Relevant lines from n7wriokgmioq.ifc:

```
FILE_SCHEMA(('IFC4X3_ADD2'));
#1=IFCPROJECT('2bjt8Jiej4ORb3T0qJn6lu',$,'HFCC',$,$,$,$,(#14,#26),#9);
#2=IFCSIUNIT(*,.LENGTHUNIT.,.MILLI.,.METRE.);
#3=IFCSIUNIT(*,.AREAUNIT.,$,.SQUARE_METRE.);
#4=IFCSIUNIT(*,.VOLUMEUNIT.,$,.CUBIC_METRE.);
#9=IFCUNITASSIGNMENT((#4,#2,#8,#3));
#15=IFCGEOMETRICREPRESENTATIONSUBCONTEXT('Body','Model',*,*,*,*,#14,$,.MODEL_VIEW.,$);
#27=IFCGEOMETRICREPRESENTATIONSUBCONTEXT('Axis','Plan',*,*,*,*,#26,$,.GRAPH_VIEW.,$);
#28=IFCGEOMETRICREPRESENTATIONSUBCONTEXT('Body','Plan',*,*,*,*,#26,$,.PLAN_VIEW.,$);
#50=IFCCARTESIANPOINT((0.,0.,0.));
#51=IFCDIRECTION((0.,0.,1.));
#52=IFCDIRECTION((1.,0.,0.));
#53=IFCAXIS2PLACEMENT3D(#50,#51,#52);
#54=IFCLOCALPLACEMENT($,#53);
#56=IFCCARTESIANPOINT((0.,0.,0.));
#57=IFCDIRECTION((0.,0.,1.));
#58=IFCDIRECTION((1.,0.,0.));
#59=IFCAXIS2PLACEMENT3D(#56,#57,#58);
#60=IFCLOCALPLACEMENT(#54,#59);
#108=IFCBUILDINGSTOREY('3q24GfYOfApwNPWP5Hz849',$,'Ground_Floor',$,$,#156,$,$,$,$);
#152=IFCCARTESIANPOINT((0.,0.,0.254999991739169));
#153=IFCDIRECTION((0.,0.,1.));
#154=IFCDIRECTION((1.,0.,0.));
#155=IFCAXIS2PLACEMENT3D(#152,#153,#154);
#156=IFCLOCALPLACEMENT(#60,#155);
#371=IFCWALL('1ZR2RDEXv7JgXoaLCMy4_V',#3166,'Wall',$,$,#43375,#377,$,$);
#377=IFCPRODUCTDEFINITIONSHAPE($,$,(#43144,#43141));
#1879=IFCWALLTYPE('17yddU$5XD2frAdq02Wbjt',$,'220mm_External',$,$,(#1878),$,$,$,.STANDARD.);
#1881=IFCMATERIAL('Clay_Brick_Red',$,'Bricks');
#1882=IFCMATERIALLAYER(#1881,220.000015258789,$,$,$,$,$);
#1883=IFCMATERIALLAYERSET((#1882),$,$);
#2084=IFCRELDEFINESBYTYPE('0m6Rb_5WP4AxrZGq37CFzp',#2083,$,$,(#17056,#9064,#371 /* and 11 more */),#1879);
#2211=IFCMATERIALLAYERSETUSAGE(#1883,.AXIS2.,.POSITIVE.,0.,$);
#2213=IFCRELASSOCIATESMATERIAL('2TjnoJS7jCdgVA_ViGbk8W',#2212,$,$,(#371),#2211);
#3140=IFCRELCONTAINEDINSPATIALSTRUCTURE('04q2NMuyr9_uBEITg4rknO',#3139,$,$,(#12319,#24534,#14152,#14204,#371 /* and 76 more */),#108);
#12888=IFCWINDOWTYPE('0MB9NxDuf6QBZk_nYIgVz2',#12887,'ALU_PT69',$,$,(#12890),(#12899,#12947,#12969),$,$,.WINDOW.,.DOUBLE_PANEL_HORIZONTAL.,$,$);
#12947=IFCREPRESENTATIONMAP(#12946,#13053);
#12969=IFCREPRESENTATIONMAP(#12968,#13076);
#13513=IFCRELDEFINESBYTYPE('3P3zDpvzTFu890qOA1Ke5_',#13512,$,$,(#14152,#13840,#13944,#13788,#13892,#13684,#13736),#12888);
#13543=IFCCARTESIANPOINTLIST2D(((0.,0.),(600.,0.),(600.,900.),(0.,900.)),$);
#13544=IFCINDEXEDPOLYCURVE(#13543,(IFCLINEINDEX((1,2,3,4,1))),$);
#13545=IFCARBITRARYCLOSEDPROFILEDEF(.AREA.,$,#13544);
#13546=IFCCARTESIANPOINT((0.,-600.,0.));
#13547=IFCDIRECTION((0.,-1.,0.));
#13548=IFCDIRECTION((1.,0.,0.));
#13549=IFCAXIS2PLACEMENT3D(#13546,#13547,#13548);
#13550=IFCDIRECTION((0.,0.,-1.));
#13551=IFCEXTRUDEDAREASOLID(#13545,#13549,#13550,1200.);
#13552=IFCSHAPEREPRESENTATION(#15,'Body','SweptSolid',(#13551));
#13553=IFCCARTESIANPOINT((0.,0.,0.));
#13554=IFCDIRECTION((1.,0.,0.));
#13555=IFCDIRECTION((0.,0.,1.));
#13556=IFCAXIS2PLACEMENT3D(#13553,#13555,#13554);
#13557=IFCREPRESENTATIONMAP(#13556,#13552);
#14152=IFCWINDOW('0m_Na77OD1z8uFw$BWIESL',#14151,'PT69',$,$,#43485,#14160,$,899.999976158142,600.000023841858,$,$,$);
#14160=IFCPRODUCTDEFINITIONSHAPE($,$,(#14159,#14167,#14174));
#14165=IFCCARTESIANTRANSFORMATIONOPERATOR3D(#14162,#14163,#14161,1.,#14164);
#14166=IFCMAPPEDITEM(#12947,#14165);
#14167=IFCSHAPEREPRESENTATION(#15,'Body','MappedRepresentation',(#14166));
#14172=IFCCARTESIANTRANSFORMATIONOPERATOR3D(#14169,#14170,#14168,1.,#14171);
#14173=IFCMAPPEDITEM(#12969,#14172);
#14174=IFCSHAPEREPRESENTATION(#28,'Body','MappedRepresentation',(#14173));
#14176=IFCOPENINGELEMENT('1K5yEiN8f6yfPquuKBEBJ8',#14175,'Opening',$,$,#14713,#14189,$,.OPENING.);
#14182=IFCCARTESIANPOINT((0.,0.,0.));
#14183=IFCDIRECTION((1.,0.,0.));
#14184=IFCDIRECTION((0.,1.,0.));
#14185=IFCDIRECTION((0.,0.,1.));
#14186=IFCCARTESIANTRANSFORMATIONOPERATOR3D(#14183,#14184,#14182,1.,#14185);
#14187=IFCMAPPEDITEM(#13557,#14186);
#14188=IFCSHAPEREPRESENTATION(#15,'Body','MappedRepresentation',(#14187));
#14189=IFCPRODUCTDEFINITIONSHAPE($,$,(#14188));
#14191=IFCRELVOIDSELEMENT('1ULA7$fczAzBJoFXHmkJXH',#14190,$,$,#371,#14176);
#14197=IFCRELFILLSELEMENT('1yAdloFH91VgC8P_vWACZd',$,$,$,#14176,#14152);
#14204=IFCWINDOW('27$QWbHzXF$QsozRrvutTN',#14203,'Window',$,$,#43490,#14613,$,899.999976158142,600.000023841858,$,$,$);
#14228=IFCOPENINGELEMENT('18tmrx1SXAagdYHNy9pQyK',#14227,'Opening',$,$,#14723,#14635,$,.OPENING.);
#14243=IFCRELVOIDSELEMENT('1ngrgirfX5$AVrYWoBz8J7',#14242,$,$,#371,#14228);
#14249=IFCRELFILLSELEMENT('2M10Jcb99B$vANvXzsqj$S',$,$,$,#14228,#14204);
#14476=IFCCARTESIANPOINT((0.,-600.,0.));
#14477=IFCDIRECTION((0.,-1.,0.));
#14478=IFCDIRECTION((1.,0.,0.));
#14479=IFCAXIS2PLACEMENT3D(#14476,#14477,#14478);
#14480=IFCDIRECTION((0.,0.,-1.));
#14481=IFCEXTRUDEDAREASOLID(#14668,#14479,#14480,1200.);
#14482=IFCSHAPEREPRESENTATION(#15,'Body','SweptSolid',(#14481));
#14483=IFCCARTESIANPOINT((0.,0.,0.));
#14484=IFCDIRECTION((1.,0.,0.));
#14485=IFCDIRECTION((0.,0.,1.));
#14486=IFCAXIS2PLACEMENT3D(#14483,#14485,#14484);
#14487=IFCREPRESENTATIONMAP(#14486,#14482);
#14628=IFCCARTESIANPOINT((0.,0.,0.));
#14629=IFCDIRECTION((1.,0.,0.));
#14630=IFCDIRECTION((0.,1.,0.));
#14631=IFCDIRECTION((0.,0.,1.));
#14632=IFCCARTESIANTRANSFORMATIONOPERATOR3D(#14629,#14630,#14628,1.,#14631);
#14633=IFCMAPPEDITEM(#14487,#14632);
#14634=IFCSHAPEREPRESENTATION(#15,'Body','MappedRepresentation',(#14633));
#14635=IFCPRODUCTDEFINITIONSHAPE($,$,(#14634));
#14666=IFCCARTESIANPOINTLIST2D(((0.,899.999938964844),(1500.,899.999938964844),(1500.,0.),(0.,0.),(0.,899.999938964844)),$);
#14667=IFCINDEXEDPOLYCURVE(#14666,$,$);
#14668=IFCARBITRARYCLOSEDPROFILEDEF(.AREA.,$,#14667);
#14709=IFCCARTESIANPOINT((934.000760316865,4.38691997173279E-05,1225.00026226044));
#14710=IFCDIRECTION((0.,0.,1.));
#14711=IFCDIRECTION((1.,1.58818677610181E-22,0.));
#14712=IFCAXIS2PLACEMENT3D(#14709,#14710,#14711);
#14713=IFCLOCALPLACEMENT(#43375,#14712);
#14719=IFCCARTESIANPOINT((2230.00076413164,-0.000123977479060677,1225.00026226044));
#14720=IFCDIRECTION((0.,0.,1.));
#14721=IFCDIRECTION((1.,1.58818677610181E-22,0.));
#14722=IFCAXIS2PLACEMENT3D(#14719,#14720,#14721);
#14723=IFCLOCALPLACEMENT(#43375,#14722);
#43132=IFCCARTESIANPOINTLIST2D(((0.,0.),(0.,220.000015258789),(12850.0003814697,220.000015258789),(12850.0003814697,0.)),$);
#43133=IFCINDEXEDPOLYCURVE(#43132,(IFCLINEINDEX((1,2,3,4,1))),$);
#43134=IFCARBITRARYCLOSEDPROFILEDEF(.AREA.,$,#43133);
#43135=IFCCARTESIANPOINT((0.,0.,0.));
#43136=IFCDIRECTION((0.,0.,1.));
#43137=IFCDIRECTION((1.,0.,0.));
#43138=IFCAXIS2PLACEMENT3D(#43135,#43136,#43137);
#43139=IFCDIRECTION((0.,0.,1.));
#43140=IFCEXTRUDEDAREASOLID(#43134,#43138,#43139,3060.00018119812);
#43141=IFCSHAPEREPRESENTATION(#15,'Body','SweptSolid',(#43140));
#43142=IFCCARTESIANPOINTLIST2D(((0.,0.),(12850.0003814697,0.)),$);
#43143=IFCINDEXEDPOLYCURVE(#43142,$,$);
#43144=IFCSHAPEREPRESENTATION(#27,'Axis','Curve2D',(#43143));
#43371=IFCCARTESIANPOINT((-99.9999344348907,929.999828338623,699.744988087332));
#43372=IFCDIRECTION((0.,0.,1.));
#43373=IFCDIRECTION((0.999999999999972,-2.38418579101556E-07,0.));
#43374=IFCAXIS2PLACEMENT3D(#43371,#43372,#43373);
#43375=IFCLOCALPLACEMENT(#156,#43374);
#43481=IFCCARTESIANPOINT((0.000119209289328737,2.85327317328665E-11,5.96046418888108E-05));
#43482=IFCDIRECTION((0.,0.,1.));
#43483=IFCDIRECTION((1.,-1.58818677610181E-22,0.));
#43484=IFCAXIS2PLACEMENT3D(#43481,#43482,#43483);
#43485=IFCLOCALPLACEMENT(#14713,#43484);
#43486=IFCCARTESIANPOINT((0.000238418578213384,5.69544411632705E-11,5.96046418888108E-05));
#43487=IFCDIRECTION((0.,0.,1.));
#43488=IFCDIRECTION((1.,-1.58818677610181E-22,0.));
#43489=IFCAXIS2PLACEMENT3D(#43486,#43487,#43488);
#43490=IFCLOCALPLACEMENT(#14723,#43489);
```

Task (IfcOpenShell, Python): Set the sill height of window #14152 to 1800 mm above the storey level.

```python
import numpy as np
import ifcopenshell
import ifcopenshell.api.geometry
import ifcopenshell.geom
import ifcopenshell.util.element
import ifcopenshell.util.placement
import ifcopenshell.util.shape
import ifcopenshell.util.unit

model = ifcopenshell.open("n7wriokgmioq.ifc")
unit_scale = ifcopenshell.util.unit.calculate_unit_scale(model)

window = model.by_guid("0m_Na77OD1z8uFw$BWIESL")
opening = window.FillsVoids[0].RelatingOpeningElement
storey = ifcopenshell.util.element.get_container(window, ifc_class="IfcBuildingStorey")
level = ifcopenshell.util.placement.get_local_placement(storey.ObjectPlacement)[2, 3]

# The opening's origin need not be at the sill, so measure its lowest point.
shape = ifcopenshell.geom.create_shape(ifcopenshell.geom.settings(), opening)
bottom = ifcopenshell.util.shape.get_shape_bottom_elevation(shape, shape.geometry) / unit_scale
dz = level + 1.8 / unit_scale - bottom

shift = np.array([0.0, 0.0, dz])
# The window is placed relative to its opening, so it follows when the opening moves.
matrix = ifcopenshell.util.placement.get_local_placement(opening.ObjectPlacement)
matrix[:3, 3] += shift
ifcopenshell.api.geometry.edit_object_placement(
    model, product=opening, matrix=matrix, is_si=False, should_transform_children=True
)

print(f"moved by {dz * unit_scale:+.3f} m")

model.write("n7wriokgmioq_updated.ifc")
```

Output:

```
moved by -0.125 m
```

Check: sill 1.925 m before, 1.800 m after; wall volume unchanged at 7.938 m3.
